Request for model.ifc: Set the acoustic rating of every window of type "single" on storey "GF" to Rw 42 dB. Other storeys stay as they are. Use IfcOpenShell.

First a look at what the model holds.

```python
import ifcopenshell
import ifcopenshell.util.element

model = ifcopenshell.open("model.ifc")
print(model.schema)
storey = next(s for s in model.by_type("IfcBuildingStorey") if s.Name == "GF")
windows = [e for e in ifcopenshell.util.element.get_decomposition(storey) if e.is_a("IfcWindow")]
seen = {}
for e in windows:
    element_type = ifcopenshell.util.element.get_type(e)
    key = (element_type.Name if element_type != e and element_type else None, ifcopenshell.util.element.get_pset(e, "Pset_WindowCommon", "AcousticRating"))
    seen[key] = seen.get(key, 0) + 1
for (name, value), count in sorted(seen.items(), key=str):
    print(count, "x", name, "|", value)
```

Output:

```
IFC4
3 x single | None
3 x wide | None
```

```python
import ifcopenshell
import ifcopenshell.api.pset
import ifcopenshell.util.element

model = ifcopenshell.open("model.ifc")

storey = next(s for s in model.by_type("IfcBuildingStorey") if s.Name == "GF")
windows = [e for e in ifcopenshell.util.element.get_decomposition(storey) if e.is_a("IfcWindow")]

count = 0
for e in windows:
    element_type = ifcopenshell.util.element.get_type(e)
    if element_type in (None, e) or element_type.Name != "single":
        continue
    # add_pset returns the element's existing set when there is one.
    pset = ifcopenshell.api.pset.add_pset(model, product=e, name="Pset_WindowCommon")
    ifcopenshell.api.pset.edit_pset(model, pset=pset, properties={"AcousticRating": "Rw 42 dB"})
    count += 1

print(count, "windows updated")

model.write("model_edited.ifc")
```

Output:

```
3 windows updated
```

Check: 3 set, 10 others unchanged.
